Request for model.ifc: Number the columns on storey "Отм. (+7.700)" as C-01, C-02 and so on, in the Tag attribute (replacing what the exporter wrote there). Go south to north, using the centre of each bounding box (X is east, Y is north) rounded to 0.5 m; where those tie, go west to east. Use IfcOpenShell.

First a look at what the model holds.

```python
import ifcopenshell
import ifcopenshell.util.element
import ifcopenshell.util.placement

model = ifcopenshell.open("model.ifc")
print(model.schema)
storey = next(s for s in model.by_type("IfcBuildingStorey") if s.Name == "Отм. (+7.700)")
columns = [e for e in ifcopenshell.util.element.get_decomposition(storey) if e.is_a("IfcColumn")]
for e in sorted(columns, key=lambda e: e.id()):
    origin = ifcopenshell.util.placement.get_local_placement(e.ObjectPlacement)[:3, 3]
    print(e.id(), e.Tag, e.Name, origin.round(2) + 0.0, sep=" | ")
```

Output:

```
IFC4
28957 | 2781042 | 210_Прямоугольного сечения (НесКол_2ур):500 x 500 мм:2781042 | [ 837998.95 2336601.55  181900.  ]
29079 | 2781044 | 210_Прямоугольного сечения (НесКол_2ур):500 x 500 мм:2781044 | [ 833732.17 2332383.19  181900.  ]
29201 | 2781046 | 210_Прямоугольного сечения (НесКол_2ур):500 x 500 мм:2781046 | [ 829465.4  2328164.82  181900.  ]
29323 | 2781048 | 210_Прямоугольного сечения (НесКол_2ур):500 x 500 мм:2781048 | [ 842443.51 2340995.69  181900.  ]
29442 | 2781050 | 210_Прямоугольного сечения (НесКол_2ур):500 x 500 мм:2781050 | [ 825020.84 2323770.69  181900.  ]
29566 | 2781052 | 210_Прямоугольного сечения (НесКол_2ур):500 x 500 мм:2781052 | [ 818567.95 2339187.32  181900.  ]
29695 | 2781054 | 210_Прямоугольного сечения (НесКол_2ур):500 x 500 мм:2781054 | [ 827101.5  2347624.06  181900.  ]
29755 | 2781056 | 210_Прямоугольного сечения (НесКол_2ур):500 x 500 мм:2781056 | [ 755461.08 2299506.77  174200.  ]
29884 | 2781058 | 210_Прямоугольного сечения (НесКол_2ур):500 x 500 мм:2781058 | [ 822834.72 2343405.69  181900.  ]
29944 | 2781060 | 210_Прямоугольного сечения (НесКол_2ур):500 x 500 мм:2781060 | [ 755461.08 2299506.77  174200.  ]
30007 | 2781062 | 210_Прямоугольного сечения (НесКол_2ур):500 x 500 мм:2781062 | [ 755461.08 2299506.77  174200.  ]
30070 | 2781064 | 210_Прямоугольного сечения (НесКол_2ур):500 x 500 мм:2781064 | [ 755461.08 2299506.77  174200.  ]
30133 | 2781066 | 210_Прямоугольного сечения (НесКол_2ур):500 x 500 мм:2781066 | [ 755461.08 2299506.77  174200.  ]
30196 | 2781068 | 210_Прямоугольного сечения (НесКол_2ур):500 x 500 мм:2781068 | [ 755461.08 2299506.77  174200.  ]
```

```python
import ifcopenshell
import ifcopenshell.geom
import ifcopenshell.util.element
import ifcopenshell.util.shape

model = ifcopenshell.open("model.ifc")
settings = ifcopenshell.geom.settings()
settings.set("use-world-coords", True)


def centre(element):
    shape = ifcopenshell.geom.create_shape(settings, element)
    return ifcopenshell.util.shape.get_bbox_centroid(shape.geometry)


storey = next(s for s in model.by_type("IfcBuildingStorey") if s.Name == "Отм. (+7.700)")
columns = [e for e in ifcopenshell.util.element.get_decomposition(storey) if e.is_a("IfcColumn")]

# Insertion points can sit at a corner or the storey origin, so sort by the geometry (in metres).
centres = {e: centre(e) for e in columns}
columns.sort(key=lambda e: (round(centres[e][1] / 0.5), centres[e][0]))

for i, e in enumerate(columns, start=1):
    number = f"C-{i:02d}"
    e.Tag = number
    print(e.id(), number)

model.write("model-out.ifc")
```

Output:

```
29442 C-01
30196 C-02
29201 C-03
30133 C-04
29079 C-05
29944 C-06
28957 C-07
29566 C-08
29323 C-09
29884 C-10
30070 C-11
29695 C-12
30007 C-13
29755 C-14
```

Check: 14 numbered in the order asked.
